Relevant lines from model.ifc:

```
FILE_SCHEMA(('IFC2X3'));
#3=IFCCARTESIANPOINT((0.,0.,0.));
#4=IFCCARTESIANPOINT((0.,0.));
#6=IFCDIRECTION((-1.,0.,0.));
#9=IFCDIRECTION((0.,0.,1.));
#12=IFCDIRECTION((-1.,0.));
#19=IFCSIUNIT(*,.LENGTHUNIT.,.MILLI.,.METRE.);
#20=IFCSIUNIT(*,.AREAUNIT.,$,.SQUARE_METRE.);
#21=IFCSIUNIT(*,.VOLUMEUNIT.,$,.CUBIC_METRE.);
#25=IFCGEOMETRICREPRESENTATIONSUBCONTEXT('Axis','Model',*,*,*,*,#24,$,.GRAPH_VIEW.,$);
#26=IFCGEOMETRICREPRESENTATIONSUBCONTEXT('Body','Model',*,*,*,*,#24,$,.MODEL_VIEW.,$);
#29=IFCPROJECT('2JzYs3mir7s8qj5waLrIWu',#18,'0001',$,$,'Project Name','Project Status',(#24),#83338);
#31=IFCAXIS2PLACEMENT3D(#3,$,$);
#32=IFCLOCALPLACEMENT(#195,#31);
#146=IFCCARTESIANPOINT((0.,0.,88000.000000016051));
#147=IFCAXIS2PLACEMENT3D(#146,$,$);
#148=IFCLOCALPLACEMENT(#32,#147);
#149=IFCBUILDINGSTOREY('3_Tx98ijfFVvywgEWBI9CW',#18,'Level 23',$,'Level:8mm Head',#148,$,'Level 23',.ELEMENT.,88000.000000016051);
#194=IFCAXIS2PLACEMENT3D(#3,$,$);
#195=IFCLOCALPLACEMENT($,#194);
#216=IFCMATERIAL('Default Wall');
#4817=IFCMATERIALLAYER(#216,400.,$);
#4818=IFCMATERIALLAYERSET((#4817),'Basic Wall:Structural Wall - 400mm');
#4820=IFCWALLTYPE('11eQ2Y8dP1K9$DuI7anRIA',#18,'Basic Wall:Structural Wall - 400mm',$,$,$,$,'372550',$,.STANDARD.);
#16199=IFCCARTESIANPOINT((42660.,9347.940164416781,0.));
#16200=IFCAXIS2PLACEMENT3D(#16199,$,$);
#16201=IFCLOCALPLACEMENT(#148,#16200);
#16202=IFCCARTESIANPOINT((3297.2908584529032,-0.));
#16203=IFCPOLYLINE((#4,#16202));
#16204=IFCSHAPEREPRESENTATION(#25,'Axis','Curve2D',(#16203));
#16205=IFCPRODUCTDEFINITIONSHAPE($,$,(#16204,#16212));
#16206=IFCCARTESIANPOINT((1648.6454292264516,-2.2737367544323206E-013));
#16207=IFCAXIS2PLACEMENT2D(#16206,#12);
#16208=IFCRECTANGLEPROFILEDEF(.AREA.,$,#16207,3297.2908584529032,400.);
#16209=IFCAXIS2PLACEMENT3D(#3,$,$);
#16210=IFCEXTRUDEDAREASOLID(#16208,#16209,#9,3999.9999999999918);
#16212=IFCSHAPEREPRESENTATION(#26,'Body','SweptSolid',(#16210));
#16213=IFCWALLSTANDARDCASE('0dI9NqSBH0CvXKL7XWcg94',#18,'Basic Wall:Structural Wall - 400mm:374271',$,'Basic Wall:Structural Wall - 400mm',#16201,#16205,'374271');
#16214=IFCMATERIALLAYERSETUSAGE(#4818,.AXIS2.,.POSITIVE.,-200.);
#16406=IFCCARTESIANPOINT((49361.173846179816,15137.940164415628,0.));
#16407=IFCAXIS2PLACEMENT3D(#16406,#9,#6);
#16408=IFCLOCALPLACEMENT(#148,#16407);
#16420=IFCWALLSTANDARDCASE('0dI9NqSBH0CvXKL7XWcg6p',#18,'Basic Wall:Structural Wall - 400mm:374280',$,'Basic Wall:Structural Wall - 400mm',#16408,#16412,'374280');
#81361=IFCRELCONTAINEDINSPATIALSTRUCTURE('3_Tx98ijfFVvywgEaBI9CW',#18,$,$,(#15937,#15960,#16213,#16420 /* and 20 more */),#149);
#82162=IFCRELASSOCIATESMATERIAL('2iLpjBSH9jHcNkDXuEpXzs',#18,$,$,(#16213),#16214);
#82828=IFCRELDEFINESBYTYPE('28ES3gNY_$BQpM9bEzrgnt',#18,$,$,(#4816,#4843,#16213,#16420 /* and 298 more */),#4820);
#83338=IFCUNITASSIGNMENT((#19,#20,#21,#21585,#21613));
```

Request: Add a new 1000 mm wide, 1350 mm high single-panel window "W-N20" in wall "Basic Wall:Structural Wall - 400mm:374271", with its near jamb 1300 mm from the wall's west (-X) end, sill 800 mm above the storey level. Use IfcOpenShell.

```python
import numpy as np
import ifcopenshell
import ifcopenshell.api.feature
import ifcopenshell.api.geometry
import ifcopenshell.api.root
import ifcopenshell.api.spatial
import ifcopenshell.api.type
import ifcopenshell.geom
import ifcopenshell.util.element
import ifcopenshell.util.placement
import ifcopenshell.util.representation
import ifcopenshell.util.shape
import ifcopenshell.util.unit

model = ifcopenshell.open("model.ifc")
unit_scale = ifcopenshell.util.unit.calculate_unit_scale(model)
settings = ifcopenshell.geom.settings()


def volume(element):
    """Net volume in cubic metres, openings subtracted."""
    shape = ifcopenshell.geom.create_shape(settings, element)
    return ifcopenshell.util.shape.get_volume(shape.geometry)


wall = model.by_guid("0dI9NqSBH0CvXKL7XWcg94")
storey = ifcopenshell.util.element.get_container(wall, ifc_class="IfcBuildingStorey")
context = ifcopenshell.util.representation.get_context(model, "Model", "Body", "MODEL_VIEW")
before = volume(wall)

width, height, from_end, sill = 1, 1.35, 1.3, 0.8  # metres

# The wall runs along its own X axis, and the end named is its -X end.
wall_shape = ifcopenshell.geom.create_shape(settings, wall)
x, y, z = ifcopenshell.util.shape.get_vertices(wall_shape.geometry).T
start = x.min() + from_end
face, thickness = float(y.min()), float(y.max() - y.min())
wall_matrix = ifcopenshell.util.placement.get_local_placement(wall.ObjectPlacement)
level = ifcopenshell.util.placement.get_local_placement(storey.ObjectPlacement)[2, 3]


def in_wall(x, y):
    """Placement at x, y metres in the wall's axes, at sill height."""
    matrix = wall_matrix.copy()
    matrix[:, 3] = wall_matrix @ np.array([x / unit_scale, y / unit_scale, 0.0, 1.0])
    matrix[2, 3] = level + sill / unit_scale
    return matrix


# Opening: a box that overshoots both wall faces by 50 mm.
opening = ifcopenshell.api.root.create_entity(model, ifc_class="IfcOpeningElement")
box = ifcopenshell.api.geometry.add_wall_representation(
    model, context=context, length=width, height=height, thickness=thickness + 0.1
)
ifcopenshell.api.geometry.assign_representation(model, product=opening, representation=box)
ifcopenshell.api.geometry.edit_object_placement(model, product=opening, matrix=in_wall(start, face - 0.05), is_si=False)
ifcopenshell.api.feature.add_feature(model, feature=opening, element=wall)

window = ifcopenshell.api.root.create_entity(model, ifc_class="IfcWindow", name="W-N20")
window.OverallWidth, window.OverallHeight = width / unit_scale, height / unit_scale
body = ifcopenshell.api.geometry.add_window_representation(
    model,
    context=context,
    overall_width=window.OverallWidth,
    overall_height=window.OverallHeight,
    partition_type="SINGLE_PANEL",
)
ifcopenshell.api.geometry.assign_representation(model, product=window, representation=body)
ifcopenshell.api.spatial.assign_container(model, products=[window], relating_structure=storey)
fills = ifcopenshell.api.feature.add_filling(model, opening=opening, element=window)
fills.OwnerHistory = window.OwnerHistory  # required in IFC2X3

# IFC2X3 keeps the operation on the window style.
style = ifcopenshell.api.root.create_entity(model, ifc_class="IfcWindowStyle", name="W-N20")
style.OperationType, style.ConstructionType = "SINGLE_PANEL", "NOTDEFINED"
style.ParameterTakesPrecedence = style.Sizeable = False
ifcopenshell.api.type.assign_type(model, related_objects=[window], relating_type=style)

# Centre the window in the wall's thickness.
ifcopenshell.api.geometry.edit_object_placement(model, product=window, matrix=in_wall(start, face), is_si=False)
window_shape = ifcopenshell.geom.create_shape(settings, window)
depth = ifcopenshell.util.shape.get_vertices(window_shape.geometry)[:, 1]
offset = face + thickness / 2 - (depth.min() + depth.max()) / 2
ifcopenshell.api.geometry.edit_object_placement(model, product=window, matrix=in_wall(start, offset), is_si=False)

after = volume(wall)

print(f"wall volume {before:.3f} -> {after:.3f} m3")

model.write("model_v2.ifc")
```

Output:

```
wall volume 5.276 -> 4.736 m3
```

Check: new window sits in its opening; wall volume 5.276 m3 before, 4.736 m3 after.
